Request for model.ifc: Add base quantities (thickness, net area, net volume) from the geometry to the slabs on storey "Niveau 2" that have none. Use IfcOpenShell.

First a look at what the model holds.

```python
import ifcopenshell
import ifcopenshell.util.element
import ifcopenshell.util.unit

model = ifcopenshell.open("model.ifc")
print(model.schema)
for unit_type in ("LENGTHUNIT", "AREAUNIT", "VOLUMEUNIT"):
    print(unit_type, ifcopenshell.util.unit.calculate_unit_scale(model, unit_type))
storey = next(s for s in model.by_type("IfcBuildingStorey") if s.Name == "Niveau 2")
slabs = [e for e in ifcopenshell.util.element.get_decomposition(storey) if e.is_a("IfcSlab")]
for e in sorted(slabs, key=lambda e: e.id()):
    print(e.id(), e.is_a(), e.Name, list(ifcopenshell.util.element.get_psets(e, qtos_only=True)), sep=" | ")
```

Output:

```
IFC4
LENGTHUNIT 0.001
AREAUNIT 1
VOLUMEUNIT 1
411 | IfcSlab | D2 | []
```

```python
import ifcopenshell
import ifcopenshell.api.pset
import ifcopenshell.geom
import ifcopenshell.util.element
import ifcopenshell.util.shape
import ifcopenshell.util.unit

model = ifcopenshell.open("model.ifc")
unit_scale = ifcopenshell.util.unit.calculate_unit_scale(model)
area_scale = ifcopenshell.util.unit.calculate_unit_scale(model, "AREAUNIT")
volume_scale = ifcopenshell.util.unit.calculate_unit_scale(model, "VOLUMEUNIT")
settings = ifcopenshell.geom.settings()

storey = next(s for s in model.by_type("IfcBuildingStorey") if s.Name == "Niveau 2")
slabs = [e for e in ifcopenshell.util.element.get_decomposition(storey) if e.is_a("IfcSlab")]

for e in sorted(slabs, key=lambda e: e.id()):
    if ifcopenshell.util.element.get_psets(e, qtos_only=True, should_inherit=False):
        continue
    # Geometry comes back in metres, in the element's own axes.
    shape = ifcopenshell.geom.create_shape(settings, e)
    values = {
        "Width": ifcopenshell.util.shape.get_z(shape.geometry) / unit_scale,
        "NetArea": ifcopenshell.util.shape.get_footprint_area(shape.geometry) / area_scale,
        "NetVolume": ifcopenshell.util.shape.get_volume(shape.geometry) / volume_scale,
    }
    qto = ifcopenshell.api.pset.add_qto(model, product=e, name="Qto_SlabBaseQuantities")
    ifcopenshell.api.pset.edit_qto(model, qto=qto, properties=values)
    print(e.id(), {k: round(v, 3) for k, v in values.items()})

model.write("model_edited.ifc")
```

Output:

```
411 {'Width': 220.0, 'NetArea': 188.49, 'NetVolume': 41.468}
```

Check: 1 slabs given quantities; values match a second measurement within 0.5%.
